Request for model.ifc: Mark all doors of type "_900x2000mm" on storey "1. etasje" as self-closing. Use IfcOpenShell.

First a look at what the model holds.

```python
import ifcopenshell
import ifcopenshell.util.element

model = ifcopenshell.open("model.ifc")
print(model.schema)
storey = next(s for s in model.by_type("IfcBuildingStorey") if s.Name == "1. etasje")
doors = [e for e in ifcopenshell.util.element.get_decomposition(storey) if e.is_a("IfcDoor")]
seen = {}
for e in doors:
    element_type = ifcopenshell.util.element.get_type(e)
    key = (element_type.Name if element_type != e and element_type else None, ifcopenshell.util.element.get_pset(e, "Pset_DoorCommon", "SelfClosing"))
    seen[key] = seen.get(key, 0) + 1
for (name, value), count in sorted(seen.items(), key=str):
    print(count, "x", name, "|", value)
```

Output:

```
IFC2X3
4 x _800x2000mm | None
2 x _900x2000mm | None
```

```python
import ifcopenshell
import ifcopenshell.api.pset
import ifcopenshell.util.element

model = ifcopenshell.open("model.ifc")

storey = next(s for s in model.by_type("IfcBuildingStorey") if s.Name == "1. etasje")
doors = [e for e in ifcopenshell.util.element.get_decomposition(storey) if e.is_a("IfcDoor")]

count = 0
for e in doors:
    element_type = ifcopenshell.util.element.get_type(e)
    if element_type in (None, e) or element_type.Name != "_900x2000mm":
        continue
    # add_pset returns the element's existing set when there is one.
    pset = ifcopenshell.api.pset.add_pset(model, product=e, name="Pset_DoorCommon")
    ifcopenshell.api.pset.edit_pset(model, pset=pset, properties={"SelfClosing": True})
    count += 1

print(count, "doors updated")

model.write("model_rev.ifc")
```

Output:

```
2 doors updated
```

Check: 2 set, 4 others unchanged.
